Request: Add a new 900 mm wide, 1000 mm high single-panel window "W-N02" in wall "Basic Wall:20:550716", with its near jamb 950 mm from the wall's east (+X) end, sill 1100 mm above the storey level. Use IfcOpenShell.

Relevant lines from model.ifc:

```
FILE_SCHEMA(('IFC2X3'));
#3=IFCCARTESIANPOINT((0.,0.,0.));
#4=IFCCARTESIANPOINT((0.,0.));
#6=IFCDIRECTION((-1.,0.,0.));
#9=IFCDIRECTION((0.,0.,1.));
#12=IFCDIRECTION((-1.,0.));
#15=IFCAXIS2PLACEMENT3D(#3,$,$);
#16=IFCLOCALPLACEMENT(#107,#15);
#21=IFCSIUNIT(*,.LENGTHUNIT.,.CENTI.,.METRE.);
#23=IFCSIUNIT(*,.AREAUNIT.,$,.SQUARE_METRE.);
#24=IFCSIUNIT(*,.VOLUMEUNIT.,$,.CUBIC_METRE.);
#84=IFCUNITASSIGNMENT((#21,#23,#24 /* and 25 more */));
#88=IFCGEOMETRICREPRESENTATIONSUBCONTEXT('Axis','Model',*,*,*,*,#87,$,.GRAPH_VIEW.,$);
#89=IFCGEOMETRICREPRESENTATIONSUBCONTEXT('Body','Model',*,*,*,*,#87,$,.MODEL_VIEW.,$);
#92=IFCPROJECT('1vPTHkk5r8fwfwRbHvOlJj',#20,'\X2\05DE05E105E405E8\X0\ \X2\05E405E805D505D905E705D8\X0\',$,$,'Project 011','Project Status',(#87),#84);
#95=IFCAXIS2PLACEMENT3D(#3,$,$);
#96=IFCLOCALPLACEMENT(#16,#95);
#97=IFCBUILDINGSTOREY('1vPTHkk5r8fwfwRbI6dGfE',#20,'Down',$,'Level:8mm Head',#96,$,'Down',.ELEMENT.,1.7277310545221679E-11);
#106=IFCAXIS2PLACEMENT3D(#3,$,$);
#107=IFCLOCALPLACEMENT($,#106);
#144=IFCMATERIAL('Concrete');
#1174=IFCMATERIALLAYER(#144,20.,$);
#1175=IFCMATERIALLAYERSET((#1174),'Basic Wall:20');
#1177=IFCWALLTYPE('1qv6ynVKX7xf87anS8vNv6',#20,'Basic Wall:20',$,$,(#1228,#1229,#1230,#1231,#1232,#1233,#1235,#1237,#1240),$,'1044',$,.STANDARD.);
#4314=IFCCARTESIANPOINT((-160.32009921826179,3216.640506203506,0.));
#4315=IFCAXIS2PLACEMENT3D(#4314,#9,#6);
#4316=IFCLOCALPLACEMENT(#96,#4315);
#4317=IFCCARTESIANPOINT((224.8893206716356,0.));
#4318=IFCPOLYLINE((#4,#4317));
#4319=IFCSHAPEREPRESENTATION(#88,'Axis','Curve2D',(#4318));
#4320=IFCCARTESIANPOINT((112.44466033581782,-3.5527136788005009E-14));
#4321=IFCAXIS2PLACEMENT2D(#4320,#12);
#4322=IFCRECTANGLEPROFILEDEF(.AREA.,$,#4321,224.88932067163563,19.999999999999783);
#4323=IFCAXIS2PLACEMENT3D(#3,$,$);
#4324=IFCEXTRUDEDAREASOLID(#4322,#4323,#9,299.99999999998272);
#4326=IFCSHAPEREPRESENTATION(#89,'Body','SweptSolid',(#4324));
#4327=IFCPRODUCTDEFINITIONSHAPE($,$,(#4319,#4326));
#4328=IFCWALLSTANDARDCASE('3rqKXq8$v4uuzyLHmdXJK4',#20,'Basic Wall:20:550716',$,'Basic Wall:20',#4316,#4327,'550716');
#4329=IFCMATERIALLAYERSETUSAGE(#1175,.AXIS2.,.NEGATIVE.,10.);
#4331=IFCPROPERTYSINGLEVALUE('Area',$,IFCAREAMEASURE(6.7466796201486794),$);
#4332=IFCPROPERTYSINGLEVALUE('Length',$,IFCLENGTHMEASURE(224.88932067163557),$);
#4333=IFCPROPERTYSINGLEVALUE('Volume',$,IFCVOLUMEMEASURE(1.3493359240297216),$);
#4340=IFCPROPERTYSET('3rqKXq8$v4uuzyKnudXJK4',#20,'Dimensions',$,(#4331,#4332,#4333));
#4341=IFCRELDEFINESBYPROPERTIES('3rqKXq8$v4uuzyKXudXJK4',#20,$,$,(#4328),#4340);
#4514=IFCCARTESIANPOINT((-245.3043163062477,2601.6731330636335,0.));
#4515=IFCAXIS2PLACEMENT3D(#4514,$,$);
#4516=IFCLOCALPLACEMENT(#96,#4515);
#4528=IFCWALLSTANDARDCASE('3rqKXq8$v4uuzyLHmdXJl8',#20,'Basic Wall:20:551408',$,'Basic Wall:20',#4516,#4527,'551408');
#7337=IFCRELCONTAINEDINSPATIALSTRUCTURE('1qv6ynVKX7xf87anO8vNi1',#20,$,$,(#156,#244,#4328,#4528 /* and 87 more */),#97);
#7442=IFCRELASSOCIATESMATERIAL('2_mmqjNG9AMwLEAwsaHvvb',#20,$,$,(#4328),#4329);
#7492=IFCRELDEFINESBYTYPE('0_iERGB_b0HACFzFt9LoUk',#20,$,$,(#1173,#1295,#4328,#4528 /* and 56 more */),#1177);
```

```python
import numpy as np
import ifcopenshell
import ifcopenshell.api.feature
import ifcopenshell.api.geometry
import ifcopenshell.api.pset
import ifcopenshell.api.root
import ifcopenshell.api.spatial
import ifcopenshell.api.type
import ifcopenshell.geom
import ifcopenshell.util.element
import ifcopenshell.util.placement
import ifcopenshell.util.representation
import ifcopenshell.util.shape
import ifcopenshell.util.unit

model = ifcopenshell.open("model.ifc")
unit_scale = ifcopenshell.util.unit.calculate_unit_scale(model)
area_scale = ifcopenshell.util.unit.calculate_unit_scale(model, "AREAUNIT")
volume_scale = ifcopenshell.util.unit.calculate_unit_scale(model, "VOLUMEUNIT")
settings = ifcopenshell.geom.settings()


def volume(element):
    """Net volume in cubic metres, openings subtracted."""
    shape = ifcopenshell.geom.create_shape(settings, element)
    return ifcopenshell.util.shape.get_volume(shape.geometry)


wall = model.by_guid("3rqKXq8$v4uuzyLHmdXJK4")
storey = ifcopenshell.util.element.get_container(wall, ifc_class="IfcBuildingStorey")
context = ifcopenshell.util.representation.get_context(model, "Model", "Body", "MODEL_VIEW")
before = volume(wall)

width, height, from_end, sill = 0.9, 1, 0.95, 1.1  # metres

# The wall runs along its own X axis, and the end named is its -X end.
wall_shape = ifcopenshell.geom.create_shape(settings, wall)
x, y, z = ifcopenshell.util.shape.get_vertices(wall_shape.geometry).T
start = x.min() + from_end
face, thickness = float(y.min()), float(y.max() - y.min())
wall_matrix = ifcopenshell.util.placement.get_local_placement(wall.ObjectPlacement)
level = ifcopenshell.util.placement.get_local_placement(storey.ObjectPlacement)[2, 3]


def in_wall(x, y):
    """Placement at x, y metres in the wall's axes, at sill height."""
    matrix = wall_matrix.copy()
    matrix[:, 3] = wall_matrix @ np.array([x / unit_scale, y / unit_scale, 0.0, 1.0])
    matrix[2, 3] = level + sill / unit_scale
    return matrix


# Opening: a box that overshoots both wall faces by 50 mm.
opening = ifcopenshell.api.root.create_entity(model, ifc_class="IfcOpeningElement")
box = ifcopenshell.api.geometry.add_wall_representation(
    model, context=context, length=width, height=height, thickness=thickness + 0.1
)
ifcopenshell.api.geometry.assign_representation(model, product=opening, representation=box)
ifcopenshell.api.geometry.edit_object_placement(model, product=opening, matrix=in_wall(start, face - 0.05), is_si=False)
ifcopenshell.api.feature.add_feature(model, feature=opening, element=wall)

window = ifcopenshell.api.root.create_entity(model, ifc_class="IfcWindow", name="W-N02")
window.OverallWidth, window.OverallHeight = width / unit_scale, height / unit_scale
body = ifcopenshell.api.geometry.add_window_representation(
    model,
    context=context,
    overall_width=window.OverallWidth,
    overall_height=window.OverallHeight,
    partition_type="SINGLE_PANEL",
)
ifcopenshell.api.geometry.assign_representation(model, product=window, representation=body)
ifcopenshell.api.spatial.assign_container(model, products=[window], relating_structure=storey)
fills = ifcopenshell.api.feature.add_filling(model, opening=opening, element=window)
fills.OwnerHistory = window.OwnerHistory  # required in IFC2X3

# IFC2X3 keeps the operation on the window style.
style = ifcopenshell.api.root.create_entity(model, ifc_class="IfcWindowStyle", name="W-N02")
style.OperationType, style.ConstructionType = "SINGLE_PANEL", "NOTDEFINED"
style.ParameterTakesPrecedence = style.Sizeable = False
ifcopenshell.api.type.assign_type(model, related_objects=[window], relating_type=style)

# Centre the window in the wall's thickness.
ifcopenshell.api.geometry.edit_object_placement(model, product=window, matrix=in_wall(start, face), is_si=False)
window_shape = ifcopenshell.geom.create_shape(settings, window)
depth = ifcopenshell.util.shape.get_vertices(window_shape.geometry)[:, 1]
offset = face + thickness / 2 - (depth.min() + depth.max()) / 2
ifcopenshell.api.geometry.edit_object_placement(model, product=window, matrix=in_wall(start, offset), is_si=False)

after = volume(wall)

# Update the wall's stored quantities.
pset = model.by_id(ifcopenshell.util.element.get_pset(wall, "Dimensions", should_inherit=False)["id"])
ifcopenshell.api.pset.edit_pset(model, pset=pset, properties={
    "Area": model.create_entity("IfcAreaMeasure", after / thickness / area_scale),
    "Volume": model.create_entity("IfcVolumeMeasure", after / volume_scale),
})

print(f"wall volume {before:.3f} -> {after:.3f} m3")

model.write("model_updated.ifc")
```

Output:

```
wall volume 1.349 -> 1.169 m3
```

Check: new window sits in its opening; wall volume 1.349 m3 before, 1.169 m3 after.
